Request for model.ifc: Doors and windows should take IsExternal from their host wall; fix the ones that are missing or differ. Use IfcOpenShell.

First a look at what the model holds.

```python
import ifcopenshell
import ifcopenshell.util.element

model = ifcopenshell.open("model.ifc")
print(model.schema)
seen = {}
for e in model.by_type("IfcDoor") + model.by_type("IfcWindow"):
    if not e.FillsVoids:
        continue
    host = e.FillsVoids[0].RelatingOpeningElement.VoidsElements[0].RelatingBuildingElement
    own = ifcopenshell.util.element.get_pset(e, f"Pset_{e.is_a()[3:].removesuffix('StandardCase')}Common", "IsExternal")
    wall = ifcopenshell.util.element.get_pset(host, "Pset_WallCommon", "IsExternal")
    seen[e.is_a(), own, wall] = seen.get((e.is_a(), own, wall), 0) + 1
for (cls, own, wall), count in sorted(seen.items(), key=str):
    print(count, cls, "IsExternal:", own, "| host wall:", wall)
```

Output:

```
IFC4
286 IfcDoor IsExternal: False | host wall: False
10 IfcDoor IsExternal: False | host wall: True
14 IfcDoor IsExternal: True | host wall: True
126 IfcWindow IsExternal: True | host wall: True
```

```python
import ifcopenshell
import ifcopenshell.api.pset
import ifcopenshell.util.element

model = ifcopenshell.open("model.ifc")

count = 0
for ifc_class, pset_name in (("IfcDoor", "Pset_DoorCommon"), ("IfcWindow", "Pset_WindowCommon")):
    for e in model.by_type(ifc_class):
        if not e.FillsVoids:
            continue
        host = e.FillsVoids[0].RelatingOpeningElement.VoidsElements[0].RelatingBuildingElement
        external = ifcopenshell.util.element.get_pset(host, "Pset_WallCommon", "IsExternal")
        if external is None or ifcopenshell.util.element.get_pset(e, pset_name, "IsExternal") == external:
            continue
        found = ifcopenshell.util.element.get_pset(e, pset_name, should_inherit=False)
        if found:
            pset = model.by_id(found["id"])
            if len(ifcopenshell.util.element.get_elements_by_pset(pset)) > 1:
                pset = ifcopenshell.api.pset.unshare_pset(model, products=[e], pset=pset)[0]
        else:
            pset = ifcopenshell.api.pset.add_pset(model, product=e, name=pset_name)
        ifcopenshell.api.pset.edit_pset(model, pset=pset, properties={"IsExternal": external})
        count += 1

print(count, "updated")

model.write("model_v2.ifc")
```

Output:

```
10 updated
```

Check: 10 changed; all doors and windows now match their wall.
